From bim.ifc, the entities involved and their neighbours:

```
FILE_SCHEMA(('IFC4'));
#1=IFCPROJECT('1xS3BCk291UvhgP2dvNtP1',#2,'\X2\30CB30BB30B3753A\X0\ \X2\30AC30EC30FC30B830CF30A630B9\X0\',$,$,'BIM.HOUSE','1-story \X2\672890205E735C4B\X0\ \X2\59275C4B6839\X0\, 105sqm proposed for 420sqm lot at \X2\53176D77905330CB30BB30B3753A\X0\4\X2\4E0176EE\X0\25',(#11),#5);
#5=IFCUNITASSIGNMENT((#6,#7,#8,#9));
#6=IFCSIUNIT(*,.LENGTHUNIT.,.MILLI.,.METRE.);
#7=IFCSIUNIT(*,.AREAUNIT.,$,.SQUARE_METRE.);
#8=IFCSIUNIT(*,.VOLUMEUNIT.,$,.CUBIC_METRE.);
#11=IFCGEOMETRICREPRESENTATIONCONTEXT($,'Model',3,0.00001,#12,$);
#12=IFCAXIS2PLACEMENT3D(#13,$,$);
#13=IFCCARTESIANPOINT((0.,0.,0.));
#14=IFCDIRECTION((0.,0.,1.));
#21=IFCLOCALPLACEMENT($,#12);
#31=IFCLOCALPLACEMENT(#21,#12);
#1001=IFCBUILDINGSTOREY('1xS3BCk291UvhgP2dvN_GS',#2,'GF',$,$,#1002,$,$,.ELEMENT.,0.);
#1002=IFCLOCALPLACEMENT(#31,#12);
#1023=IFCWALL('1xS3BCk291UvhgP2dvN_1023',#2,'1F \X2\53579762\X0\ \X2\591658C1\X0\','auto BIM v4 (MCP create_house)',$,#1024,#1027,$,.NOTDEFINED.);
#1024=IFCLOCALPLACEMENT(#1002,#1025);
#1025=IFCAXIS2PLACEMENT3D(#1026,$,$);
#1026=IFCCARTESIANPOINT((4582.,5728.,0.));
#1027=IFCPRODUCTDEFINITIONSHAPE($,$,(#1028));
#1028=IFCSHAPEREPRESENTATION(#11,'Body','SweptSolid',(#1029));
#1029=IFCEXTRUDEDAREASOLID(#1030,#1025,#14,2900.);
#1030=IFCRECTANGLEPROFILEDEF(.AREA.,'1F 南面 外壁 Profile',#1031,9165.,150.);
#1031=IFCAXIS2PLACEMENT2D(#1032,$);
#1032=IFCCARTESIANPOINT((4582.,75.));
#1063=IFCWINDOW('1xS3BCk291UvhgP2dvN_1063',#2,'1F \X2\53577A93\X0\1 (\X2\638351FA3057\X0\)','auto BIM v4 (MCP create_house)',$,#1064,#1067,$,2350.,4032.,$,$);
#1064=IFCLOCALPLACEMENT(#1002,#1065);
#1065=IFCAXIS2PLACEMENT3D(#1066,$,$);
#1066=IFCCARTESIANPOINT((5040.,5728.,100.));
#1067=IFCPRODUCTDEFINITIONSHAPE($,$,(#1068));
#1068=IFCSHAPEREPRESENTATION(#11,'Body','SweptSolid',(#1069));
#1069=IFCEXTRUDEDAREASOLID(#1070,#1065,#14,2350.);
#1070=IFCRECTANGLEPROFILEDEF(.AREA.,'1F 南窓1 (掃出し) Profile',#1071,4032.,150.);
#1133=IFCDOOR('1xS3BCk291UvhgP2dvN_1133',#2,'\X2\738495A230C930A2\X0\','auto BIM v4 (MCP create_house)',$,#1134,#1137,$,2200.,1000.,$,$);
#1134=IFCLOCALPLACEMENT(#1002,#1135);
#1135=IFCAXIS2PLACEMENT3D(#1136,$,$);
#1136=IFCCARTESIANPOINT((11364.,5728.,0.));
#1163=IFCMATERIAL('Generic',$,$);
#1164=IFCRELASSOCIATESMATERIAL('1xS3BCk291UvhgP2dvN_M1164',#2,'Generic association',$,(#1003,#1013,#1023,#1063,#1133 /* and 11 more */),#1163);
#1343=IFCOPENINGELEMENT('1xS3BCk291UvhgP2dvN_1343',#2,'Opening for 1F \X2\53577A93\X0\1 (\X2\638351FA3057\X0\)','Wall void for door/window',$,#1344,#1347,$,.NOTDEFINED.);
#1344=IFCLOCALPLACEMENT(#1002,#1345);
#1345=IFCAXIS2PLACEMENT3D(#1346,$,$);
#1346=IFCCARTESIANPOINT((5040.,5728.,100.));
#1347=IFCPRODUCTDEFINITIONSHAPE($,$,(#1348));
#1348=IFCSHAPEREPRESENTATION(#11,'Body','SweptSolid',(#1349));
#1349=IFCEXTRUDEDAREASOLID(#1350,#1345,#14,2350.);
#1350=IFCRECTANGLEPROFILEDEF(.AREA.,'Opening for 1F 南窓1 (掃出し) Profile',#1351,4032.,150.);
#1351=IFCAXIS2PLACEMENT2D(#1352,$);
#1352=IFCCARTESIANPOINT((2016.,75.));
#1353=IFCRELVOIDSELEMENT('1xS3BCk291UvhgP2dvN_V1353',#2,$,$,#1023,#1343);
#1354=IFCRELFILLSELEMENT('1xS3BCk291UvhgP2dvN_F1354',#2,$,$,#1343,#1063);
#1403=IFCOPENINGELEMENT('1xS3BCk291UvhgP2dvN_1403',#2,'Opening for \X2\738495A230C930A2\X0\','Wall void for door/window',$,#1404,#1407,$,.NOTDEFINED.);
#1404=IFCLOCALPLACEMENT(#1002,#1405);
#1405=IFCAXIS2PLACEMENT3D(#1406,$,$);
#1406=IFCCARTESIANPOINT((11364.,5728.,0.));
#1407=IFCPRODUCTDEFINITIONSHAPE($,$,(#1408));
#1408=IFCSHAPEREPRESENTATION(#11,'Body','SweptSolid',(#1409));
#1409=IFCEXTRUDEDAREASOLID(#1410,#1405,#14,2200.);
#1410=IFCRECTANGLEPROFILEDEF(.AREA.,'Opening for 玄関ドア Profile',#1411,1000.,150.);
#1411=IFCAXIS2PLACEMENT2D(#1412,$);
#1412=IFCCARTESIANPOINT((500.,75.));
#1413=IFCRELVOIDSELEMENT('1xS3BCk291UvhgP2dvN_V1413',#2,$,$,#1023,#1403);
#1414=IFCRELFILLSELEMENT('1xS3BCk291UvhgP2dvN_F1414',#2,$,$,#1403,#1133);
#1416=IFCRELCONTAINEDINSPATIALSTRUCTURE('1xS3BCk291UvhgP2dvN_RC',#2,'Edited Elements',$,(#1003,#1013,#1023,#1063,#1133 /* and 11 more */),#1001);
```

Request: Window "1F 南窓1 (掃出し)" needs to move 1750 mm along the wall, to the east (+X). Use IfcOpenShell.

```python
import ifcopenshell
import ifcopenshell.api.geometry
import ifcopenshell.util.placement
import ifcopenshell.util.unit

model = ifcopenshell.open("bim.ifc")
unit_scale = ifcopenshell.util.unit.calculate_unit_scale(model)

window = model.by_guid("1xS3BCk291UvhgP2dvN_1063")
opening = window.FillsVoids[0].RelatingOpeningElement
wall = opening.VoidsElements[0].RelatingBuildingElement

wall_matrix = ifcopenshell.util.placement.get_local_placement(wall.ObjectPlacement)
shift = wall_matrix[:3, 0] * 1.75 / unit_scale
before = ifcopenshell.util.placement.get_local_placement(window.ObjectPlacement)[:3, 3].copy()

# The window is not placed relative to its opening, so move both.
for product in (opening, window):
    matrix = ifcopenshell.util.placement.get_local_placement(product.ObjectPlacement)
    matrix[:3, 3] += shift
    ifcopenshell.api.geometry.edit_object_placement(model, product=product, matrix=matrix, is_si=False)

after = ifcopenshell.util.placement.get_local_placement(window.ObjectPlacement)[:3, 3]
print("window moved by", (after - before).round(3) + 0.0)

model.write("bim_rev.ifc")
```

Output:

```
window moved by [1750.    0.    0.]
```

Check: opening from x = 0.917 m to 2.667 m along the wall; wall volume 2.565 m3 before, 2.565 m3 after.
